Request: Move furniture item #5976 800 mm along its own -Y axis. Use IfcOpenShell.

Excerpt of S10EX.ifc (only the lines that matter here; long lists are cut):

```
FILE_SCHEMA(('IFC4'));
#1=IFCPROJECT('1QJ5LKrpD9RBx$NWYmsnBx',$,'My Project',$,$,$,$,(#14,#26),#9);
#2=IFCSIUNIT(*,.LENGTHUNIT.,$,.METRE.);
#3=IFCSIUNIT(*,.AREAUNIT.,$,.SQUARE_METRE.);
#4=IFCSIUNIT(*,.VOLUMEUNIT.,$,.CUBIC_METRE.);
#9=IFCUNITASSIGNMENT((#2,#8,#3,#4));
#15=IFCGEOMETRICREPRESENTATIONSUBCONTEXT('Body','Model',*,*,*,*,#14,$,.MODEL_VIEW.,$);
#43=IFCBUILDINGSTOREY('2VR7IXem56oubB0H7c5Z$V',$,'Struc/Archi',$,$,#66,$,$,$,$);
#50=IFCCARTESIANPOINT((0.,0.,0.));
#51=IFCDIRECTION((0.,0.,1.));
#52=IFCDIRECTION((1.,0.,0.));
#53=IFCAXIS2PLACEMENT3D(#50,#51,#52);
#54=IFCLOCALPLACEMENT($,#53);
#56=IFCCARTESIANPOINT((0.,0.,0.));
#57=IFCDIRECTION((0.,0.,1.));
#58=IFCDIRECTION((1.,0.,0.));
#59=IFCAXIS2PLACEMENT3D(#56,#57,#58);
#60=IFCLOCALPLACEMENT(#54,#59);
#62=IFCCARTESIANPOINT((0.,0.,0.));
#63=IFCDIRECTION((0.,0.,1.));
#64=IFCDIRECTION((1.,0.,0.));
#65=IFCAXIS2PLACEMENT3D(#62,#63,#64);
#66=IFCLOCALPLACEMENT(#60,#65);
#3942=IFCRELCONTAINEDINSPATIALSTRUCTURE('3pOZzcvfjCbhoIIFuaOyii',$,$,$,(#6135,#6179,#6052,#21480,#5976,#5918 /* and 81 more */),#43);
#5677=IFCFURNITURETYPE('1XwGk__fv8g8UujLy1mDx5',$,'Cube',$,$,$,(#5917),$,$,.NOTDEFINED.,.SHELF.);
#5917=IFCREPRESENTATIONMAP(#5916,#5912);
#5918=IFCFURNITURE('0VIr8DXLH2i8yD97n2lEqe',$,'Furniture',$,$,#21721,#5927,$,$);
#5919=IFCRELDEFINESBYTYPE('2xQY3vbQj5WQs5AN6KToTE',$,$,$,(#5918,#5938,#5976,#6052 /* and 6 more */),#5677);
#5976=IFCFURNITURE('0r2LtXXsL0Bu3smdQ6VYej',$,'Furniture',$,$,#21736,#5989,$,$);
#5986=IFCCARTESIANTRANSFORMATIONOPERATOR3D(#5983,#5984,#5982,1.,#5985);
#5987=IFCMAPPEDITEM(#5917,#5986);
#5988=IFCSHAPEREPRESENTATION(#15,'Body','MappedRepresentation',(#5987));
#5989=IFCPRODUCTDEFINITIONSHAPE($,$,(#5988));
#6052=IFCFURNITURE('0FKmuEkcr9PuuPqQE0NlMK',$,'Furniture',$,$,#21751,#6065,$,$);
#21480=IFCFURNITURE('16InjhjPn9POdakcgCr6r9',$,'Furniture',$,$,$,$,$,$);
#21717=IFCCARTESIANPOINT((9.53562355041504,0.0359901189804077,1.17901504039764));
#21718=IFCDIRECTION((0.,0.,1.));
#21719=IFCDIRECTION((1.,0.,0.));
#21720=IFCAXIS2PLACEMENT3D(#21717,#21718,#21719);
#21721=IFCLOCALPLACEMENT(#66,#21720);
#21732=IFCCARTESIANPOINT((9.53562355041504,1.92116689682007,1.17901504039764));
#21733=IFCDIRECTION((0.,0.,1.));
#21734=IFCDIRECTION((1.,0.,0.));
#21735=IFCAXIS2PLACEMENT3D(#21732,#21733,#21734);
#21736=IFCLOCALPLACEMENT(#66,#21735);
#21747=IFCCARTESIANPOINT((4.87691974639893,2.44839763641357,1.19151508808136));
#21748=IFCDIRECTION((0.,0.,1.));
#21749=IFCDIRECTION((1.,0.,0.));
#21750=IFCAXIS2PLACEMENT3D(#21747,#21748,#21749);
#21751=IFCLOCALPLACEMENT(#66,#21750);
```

```python
import ifcopenshell
import ifcopenshell.api.geometry
import ifcopenshell.util.placement
import ifcopenshell.util.unit

model = ifcopenshell.open("S10EX.ifc")
unit_scale = ifcopenshell.util.unit.calculate_unit_scale(model)

item = model.by_guid("0r2LtXXsL0Bu3smdQ6VYej")
matrix = ifcopenshell.util.placement.get_local_placement(item.ObjectPlacement)
matrix[:3, 3] -= matrix[:3, 1] * 0.8 / unit_scale
ifcopenshell.api.geometry.edit_object_placement(model, product=item, matrix=matrix, is_si=False)

print(ifcopenshell.util.placement.get_local_placement(item.ObjectPlacement).round(3) + 0.0)

model.write("S10EX_updated.ifc")
```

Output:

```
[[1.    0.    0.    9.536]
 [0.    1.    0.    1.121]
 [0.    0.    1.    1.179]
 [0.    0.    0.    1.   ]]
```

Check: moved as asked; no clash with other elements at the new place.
